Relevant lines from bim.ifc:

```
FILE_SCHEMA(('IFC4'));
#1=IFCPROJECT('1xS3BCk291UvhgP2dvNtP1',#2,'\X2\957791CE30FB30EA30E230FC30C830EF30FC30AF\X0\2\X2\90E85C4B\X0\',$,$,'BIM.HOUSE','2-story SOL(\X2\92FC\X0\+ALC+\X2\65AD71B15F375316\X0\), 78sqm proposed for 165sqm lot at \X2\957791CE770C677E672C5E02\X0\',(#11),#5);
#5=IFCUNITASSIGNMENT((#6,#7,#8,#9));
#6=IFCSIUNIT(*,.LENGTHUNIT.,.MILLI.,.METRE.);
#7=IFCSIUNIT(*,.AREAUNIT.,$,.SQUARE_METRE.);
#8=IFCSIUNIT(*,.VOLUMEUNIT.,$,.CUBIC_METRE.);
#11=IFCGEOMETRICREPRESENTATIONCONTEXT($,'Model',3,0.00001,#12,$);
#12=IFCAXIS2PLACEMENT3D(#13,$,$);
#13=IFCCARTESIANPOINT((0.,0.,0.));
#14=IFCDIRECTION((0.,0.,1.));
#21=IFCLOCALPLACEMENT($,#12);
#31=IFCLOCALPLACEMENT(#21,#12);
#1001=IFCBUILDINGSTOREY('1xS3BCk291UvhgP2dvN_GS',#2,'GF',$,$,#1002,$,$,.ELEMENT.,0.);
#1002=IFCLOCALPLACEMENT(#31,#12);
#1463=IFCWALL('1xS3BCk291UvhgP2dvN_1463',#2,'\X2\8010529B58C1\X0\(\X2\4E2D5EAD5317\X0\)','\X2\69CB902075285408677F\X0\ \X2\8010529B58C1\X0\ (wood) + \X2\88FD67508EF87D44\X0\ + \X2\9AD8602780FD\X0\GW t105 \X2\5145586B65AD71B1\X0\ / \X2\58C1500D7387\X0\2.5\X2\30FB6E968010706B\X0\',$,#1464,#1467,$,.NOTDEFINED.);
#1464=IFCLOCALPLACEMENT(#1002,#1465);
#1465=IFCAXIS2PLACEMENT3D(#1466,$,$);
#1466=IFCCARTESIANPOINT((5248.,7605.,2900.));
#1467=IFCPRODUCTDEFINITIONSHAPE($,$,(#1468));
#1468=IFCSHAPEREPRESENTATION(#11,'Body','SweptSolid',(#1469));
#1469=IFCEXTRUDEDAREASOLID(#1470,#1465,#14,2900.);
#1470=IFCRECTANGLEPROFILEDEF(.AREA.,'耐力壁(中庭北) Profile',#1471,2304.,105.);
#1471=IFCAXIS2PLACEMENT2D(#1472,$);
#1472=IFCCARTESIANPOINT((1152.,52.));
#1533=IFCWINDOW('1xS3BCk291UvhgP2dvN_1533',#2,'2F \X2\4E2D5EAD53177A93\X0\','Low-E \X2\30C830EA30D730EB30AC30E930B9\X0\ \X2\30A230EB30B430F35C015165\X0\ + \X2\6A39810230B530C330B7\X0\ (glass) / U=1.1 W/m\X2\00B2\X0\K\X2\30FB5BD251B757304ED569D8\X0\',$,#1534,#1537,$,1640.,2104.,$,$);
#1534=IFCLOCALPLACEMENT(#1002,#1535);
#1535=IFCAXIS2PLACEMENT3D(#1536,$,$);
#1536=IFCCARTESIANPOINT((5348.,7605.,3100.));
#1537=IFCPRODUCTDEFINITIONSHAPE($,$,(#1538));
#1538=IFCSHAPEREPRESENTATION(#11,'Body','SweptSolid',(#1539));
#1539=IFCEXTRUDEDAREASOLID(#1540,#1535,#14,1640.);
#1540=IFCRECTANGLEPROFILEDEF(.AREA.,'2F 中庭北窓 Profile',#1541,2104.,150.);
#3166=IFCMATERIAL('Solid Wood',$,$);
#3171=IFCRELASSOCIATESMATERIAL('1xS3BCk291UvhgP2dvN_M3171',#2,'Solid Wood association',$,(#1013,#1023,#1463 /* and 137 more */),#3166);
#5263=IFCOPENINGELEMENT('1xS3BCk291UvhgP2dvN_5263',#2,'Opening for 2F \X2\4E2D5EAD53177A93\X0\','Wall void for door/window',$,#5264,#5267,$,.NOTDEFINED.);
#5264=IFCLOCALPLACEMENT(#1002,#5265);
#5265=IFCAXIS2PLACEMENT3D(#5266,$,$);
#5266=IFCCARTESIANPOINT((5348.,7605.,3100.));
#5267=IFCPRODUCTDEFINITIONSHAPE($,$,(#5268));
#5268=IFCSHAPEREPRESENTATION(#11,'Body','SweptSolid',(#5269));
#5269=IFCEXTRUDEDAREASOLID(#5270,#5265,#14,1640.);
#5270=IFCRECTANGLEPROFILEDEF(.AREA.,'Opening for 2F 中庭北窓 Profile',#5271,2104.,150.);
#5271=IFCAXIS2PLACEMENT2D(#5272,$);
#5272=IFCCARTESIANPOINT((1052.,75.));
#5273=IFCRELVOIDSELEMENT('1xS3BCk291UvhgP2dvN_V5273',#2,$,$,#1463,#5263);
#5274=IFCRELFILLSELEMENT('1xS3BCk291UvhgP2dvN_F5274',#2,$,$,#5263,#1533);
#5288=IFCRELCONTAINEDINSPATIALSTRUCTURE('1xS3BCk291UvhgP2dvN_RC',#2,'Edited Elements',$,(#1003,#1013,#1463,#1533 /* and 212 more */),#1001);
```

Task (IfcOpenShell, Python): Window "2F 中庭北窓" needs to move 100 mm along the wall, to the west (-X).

```python
import ifcopenshell
import ifcopenshell.api.geometry
import ifcopenshell.util.placement
import ifcopenshell.util.unit

model = ifcopenshell.open("bim.ifc")
unit_scale = ifcopenshell.util.unit.calculate_unit_scale(model)

window = model.by_guid("1xS3BCk291UvhgP2dvN_1533")
opening = window.FillsVoids[0].RelatingOpeningElement
wall = opening.VoidsElements[0].RelatingBuildingElement

wall_matrix = ifcopenshell.util.placement.get_local_placement(wall.ObjectPlacement)
shift = wall_matrix[:3, 0] * -0.1 / unit_scale
before = ifcopenshell.util.placement.get_local_placement(window.ObjectPlacement)[:3, 3].copy()

# The window is not placed relative to its opening, so move both.
for product in (opening, window):
    matrix = ifcopenshell.util.placement.get_local_placement(product.ObjectPlacement)
    matrix[:3, 3] += shift
    ifcopenshell.api.geometry.edit_object_placement(model, product=product, matrix=matrix, is_si=False)

after = ifcopenshell.util.placement.get_local_placement(window.ObjectPlacement)[:3, 3]
print("window moved by", (after - before).round(3) + 0.0)

model.write("bim-out.ifc")
```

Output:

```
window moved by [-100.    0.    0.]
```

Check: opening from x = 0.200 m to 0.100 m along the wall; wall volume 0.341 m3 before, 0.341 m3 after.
